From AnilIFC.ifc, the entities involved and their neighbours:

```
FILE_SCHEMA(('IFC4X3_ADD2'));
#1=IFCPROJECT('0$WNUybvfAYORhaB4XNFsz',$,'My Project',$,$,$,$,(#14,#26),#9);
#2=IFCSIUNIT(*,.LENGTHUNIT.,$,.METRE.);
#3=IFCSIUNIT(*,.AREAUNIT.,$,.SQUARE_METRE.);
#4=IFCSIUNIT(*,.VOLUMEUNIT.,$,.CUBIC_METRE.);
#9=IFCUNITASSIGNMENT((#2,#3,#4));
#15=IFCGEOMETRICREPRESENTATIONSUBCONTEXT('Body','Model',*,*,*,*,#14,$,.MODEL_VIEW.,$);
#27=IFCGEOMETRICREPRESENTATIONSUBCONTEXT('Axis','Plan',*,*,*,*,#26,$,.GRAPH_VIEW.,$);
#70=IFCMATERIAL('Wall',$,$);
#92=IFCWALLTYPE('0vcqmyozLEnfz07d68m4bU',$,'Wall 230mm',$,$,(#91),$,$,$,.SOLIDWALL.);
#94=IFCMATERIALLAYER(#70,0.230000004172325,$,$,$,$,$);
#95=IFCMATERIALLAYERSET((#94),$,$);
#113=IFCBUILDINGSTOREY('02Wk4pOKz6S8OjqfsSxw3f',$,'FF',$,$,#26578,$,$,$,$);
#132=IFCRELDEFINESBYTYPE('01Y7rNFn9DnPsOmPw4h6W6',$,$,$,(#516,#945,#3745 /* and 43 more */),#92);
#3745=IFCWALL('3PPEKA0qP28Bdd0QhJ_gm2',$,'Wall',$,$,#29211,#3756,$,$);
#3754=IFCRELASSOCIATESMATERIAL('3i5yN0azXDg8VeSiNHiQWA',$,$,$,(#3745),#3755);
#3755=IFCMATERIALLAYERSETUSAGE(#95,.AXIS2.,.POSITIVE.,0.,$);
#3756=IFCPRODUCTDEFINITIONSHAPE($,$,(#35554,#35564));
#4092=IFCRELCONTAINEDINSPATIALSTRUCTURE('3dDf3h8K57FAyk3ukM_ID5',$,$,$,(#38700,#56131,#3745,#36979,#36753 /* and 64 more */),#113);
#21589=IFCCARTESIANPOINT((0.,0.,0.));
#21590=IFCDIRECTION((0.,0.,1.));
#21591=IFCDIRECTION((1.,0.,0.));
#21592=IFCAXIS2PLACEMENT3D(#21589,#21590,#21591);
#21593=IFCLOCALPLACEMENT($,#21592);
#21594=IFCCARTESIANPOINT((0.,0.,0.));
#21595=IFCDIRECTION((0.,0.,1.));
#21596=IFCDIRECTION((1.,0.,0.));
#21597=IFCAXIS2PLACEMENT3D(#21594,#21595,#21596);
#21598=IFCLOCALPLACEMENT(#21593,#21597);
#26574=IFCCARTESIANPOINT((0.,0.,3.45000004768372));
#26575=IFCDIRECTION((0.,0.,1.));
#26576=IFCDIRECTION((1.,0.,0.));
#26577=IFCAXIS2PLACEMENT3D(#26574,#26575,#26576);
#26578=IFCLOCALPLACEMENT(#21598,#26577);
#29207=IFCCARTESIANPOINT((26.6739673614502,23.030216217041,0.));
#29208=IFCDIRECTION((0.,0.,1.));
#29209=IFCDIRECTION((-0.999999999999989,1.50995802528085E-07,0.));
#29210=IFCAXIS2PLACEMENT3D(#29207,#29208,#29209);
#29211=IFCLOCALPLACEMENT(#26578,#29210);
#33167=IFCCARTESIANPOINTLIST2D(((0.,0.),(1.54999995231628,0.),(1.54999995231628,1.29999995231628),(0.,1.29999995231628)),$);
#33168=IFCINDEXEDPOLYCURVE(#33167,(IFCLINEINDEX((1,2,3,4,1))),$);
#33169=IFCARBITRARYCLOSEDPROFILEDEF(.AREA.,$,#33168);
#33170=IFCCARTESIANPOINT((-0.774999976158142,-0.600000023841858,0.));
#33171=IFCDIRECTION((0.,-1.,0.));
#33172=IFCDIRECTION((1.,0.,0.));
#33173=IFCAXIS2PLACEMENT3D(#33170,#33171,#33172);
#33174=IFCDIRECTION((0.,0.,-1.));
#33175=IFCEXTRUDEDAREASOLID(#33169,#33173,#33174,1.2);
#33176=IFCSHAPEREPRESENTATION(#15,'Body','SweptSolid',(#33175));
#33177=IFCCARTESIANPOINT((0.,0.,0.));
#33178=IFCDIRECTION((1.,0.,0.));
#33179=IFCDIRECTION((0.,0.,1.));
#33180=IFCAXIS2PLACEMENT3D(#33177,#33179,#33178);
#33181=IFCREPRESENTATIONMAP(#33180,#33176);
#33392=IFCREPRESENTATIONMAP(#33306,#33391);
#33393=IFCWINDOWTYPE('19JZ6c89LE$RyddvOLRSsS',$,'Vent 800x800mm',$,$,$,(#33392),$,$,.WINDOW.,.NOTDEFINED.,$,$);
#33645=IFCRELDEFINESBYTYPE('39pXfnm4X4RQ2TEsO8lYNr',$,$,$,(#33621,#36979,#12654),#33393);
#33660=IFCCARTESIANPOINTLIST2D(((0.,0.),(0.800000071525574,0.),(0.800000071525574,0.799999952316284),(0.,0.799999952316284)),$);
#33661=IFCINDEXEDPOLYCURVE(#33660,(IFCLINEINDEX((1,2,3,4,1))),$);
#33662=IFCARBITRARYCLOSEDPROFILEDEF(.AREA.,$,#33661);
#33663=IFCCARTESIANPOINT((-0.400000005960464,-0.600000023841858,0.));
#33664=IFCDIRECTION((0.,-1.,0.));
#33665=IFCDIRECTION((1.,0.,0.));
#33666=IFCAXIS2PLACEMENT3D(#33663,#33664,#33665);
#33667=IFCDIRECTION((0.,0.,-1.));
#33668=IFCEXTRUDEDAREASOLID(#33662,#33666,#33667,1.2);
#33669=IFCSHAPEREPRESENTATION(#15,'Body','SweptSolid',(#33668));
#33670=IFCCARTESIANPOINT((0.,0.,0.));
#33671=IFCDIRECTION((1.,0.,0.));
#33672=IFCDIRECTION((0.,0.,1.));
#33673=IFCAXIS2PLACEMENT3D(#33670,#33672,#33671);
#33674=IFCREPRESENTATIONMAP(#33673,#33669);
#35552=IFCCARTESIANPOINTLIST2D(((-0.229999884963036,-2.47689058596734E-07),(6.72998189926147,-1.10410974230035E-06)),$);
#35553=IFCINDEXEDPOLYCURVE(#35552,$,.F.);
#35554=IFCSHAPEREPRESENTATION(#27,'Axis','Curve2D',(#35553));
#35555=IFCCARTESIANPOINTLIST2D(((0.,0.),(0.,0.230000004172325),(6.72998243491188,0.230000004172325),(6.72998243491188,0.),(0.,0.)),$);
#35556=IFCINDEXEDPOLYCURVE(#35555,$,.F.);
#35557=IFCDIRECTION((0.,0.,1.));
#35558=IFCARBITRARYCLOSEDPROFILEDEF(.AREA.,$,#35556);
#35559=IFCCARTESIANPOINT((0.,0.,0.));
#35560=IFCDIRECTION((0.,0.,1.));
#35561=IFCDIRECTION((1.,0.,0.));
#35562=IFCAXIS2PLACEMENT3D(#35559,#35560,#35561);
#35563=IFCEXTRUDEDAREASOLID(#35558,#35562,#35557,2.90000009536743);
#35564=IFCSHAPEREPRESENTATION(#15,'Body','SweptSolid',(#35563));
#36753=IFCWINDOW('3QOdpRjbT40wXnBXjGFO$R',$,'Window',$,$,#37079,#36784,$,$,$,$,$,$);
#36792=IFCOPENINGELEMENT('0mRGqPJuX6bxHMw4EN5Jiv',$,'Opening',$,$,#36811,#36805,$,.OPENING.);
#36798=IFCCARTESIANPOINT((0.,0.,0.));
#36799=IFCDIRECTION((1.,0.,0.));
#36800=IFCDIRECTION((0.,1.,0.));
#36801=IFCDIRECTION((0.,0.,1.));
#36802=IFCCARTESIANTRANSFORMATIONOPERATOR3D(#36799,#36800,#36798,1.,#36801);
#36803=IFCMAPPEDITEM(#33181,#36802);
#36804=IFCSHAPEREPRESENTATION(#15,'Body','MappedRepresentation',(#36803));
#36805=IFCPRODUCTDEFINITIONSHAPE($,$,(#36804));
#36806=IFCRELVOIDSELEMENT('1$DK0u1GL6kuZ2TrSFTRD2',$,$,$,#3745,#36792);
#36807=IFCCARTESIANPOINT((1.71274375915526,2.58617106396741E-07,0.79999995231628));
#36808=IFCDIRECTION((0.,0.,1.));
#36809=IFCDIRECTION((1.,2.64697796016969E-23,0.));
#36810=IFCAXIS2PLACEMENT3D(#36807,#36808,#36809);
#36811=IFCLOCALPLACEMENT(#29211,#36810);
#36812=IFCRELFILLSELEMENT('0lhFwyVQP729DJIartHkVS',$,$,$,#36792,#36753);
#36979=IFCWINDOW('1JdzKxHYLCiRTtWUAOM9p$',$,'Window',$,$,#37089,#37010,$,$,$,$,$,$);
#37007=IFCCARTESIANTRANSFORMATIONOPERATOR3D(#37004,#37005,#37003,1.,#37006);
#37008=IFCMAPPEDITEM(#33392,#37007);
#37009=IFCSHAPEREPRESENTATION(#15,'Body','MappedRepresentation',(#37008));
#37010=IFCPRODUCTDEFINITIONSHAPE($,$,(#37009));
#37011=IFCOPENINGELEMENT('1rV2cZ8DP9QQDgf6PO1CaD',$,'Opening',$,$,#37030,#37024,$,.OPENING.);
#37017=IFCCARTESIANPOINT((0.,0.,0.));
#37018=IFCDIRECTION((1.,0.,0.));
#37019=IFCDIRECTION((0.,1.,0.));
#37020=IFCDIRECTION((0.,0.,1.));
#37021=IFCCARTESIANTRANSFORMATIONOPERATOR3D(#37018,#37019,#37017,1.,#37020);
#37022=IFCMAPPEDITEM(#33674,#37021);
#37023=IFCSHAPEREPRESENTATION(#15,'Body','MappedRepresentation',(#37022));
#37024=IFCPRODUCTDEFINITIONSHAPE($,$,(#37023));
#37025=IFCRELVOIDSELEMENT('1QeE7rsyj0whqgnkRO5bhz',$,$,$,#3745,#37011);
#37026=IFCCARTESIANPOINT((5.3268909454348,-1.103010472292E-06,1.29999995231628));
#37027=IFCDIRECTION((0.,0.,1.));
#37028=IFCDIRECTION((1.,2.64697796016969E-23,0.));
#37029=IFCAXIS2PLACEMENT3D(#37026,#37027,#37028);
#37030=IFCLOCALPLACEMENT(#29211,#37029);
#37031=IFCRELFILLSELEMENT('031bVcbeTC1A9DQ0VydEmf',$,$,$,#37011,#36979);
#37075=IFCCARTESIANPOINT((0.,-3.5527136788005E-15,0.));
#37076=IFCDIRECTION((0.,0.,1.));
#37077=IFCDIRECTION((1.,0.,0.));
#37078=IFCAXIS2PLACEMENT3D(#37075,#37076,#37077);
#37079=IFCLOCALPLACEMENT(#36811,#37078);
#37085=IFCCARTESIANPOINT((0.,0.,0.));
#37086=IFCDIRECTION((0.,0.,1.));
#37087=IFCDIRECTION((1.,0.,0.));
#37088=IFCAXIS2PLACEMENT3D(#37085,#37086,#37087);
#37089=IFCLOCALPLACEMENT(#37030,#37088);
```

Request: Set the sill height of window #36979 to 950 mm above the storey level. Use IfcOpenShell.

```python
import numpy as np
import ifcopenshell
import ifcopenshell.api.geometry
import ifcopenshell.geom
import ifcopenshell.util.element
import ifcopenshell.util.placement
import ifcopenshell.util.shape
import ifcopenshell.util.unit

model = ifcopenshell.open("AnilIFC.ifc")
unit_scale = ifcopenshell.util.unit.calculate_unit_scale(model)

window = model.by_guid("1JdzKxHYLCiRTtWUAOM9p$")
opening = window.FillsVoids[0].RelatingOpeningElement
storey = ifcopenshell.util.element.get_container(window, ifc_class="IfcBuildingStorey")
level = ifcopenshell.util.placement.get_local_placement(storey.ObjectPlacement)[2, 3]

# The opening's origin need not be at the sill, so measure its lowest point.
shape = ifcopenshell.geom.create_shape(ifcopenshell.geom.settings(), opening)
bottom = ifcopenshell.util.shape.get_shape_bottom_elevation(shape, shape.geometry) / unit_scale
dz = level + 0.95 / unit_scale - bottom

shift = np.array([0.0, 0.0, dz])
# The window is placed relative to its opening, so it follows when the opening moves.
matrix = ifcopenshell.util.placement.get_local_placement(opening.ObjectPlacement)
matrix[:3, 3] += shift
ifcopenshell.api.geometry.edit_object_placement(
    model, product=opening, matrix=matrix, is_si=False, should_transform_children=True
)

print(f"moved by {dz * unit_scale:+.3f} m")

model.write("AnilIFC_v2.ifc")
```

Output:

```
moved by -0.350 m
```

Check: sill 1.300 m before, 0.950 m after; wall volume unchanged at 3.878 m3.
